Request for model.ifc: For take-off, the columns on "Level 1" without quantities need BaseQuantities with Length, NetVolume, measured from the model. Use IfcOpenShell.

First a look at what the model holds.

```python
import ifcopenshell
import ifcopenshell.util.element
import ifcopenshell.util.unit

model = ifcopenshell.open("model.ifc")
print(model.schema)
for unit_type in ("LENGTHUNIT", "AREAUNIT", "VOLUMEUNIT"):
    print(unit_type, ifcopenshell.util.unit.calculate_unit_scale(model, unit_type))
storey = next(s for s in model.by_type("IfcBuildingStorey") if s.Name == "Level 1")
columns = [e for e in ifcopenshell.util.element.get_decomposition(storey) if e.is_a("IfcColumn")]
for e in sorted(columns, key=lambda e: e.id()):
    print(e.id(), e.is_a(), e.Name, list(ifcopenshell.util.element.get_psets(e, qtos_only=True)), sep=" | ")
```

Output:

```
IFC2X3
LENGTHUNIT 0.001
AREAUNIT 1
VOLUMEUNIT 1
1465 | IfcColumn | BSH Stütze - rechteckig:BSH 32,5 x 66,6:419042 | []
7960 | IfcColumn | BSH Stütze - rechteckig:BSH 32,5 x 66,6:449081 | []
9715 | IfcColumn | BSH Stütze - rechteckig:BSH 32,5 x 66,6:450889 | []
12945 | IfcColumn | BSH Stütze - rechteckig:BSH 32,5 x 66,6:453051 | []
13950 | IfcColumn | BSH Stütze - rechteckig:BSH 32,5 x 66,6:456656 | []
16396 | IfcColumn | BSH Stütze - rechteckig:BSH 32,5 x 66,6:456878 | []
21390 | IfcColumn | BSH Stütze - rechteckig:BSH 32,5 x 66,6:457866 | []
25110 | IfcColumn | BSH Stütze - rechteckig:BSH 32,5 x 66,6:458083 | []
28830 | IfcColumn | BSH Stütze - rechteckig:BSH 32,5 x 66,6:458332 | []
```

```python
import ifcopenshell
import ifcopenshell.api.pset
import ifcopenshell.geom
import ifcopenshell.util.element
import ifcopenshell.util.shape
import ifcopenshell.util.unit

model = ifcopenshell.open("model.ifc")
unit_scale = ifcopenshell.util.unit.calculate_unit_scale(model)
volume_scale = ifcopenshell.util.unit.calculate_unit_scale(model, "VOLUMEUNIT")
settings = ifcopenshell.geom.settings()

storey = next(s for s in model.by_type("IfcBuildingStorey") if s.Name == "Level 1")
columns = [e for e in ifcopenshell.util.element.get_decomposition(storey) if e.is_a("IfcColumn")]

for e in sorted(columns, key=lambda e: e.id()):
    if ifcopenshell.util.element.get_psets(e, qtos_only=True, should_inherit=False):
        continue
    # Geometry comes back in metres, in the element's own axes.
    shape = ifcopenshell.geom.create_shape(settings, e)
    values = {
        "Length": ifcopenshell.util.shape.get_z(shape.geometry) / unit_scale,
        "NetVolume": ifcopenshell.util.shape.get_volume(shape.geometry) / volume_scale,
    }
    qto = ifcopenshell.api.pset.add_qto(model, product=e, name="BaseQuantities")
    ifcopenshell.api.pset.edit_qto(model, qto=qto, properties=values)
    print(e.id(), {k: round(v, 3) for k, v in values.items()})

model.write("model_edited.ifc")
```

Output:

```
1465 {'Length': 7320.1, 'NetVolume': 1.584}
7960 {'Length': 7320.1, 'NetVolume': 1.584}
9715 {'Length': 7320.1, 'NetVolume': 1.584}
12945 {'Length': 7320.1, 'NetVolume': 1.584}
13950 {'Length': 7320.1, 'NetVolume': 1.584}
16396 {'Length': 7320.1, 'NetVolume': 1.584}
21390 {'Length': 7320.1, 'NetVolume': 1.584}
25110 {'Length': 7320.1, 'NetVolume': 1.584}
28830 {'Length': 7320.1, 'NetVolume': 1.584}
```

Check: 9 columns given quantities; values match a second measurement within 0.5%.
